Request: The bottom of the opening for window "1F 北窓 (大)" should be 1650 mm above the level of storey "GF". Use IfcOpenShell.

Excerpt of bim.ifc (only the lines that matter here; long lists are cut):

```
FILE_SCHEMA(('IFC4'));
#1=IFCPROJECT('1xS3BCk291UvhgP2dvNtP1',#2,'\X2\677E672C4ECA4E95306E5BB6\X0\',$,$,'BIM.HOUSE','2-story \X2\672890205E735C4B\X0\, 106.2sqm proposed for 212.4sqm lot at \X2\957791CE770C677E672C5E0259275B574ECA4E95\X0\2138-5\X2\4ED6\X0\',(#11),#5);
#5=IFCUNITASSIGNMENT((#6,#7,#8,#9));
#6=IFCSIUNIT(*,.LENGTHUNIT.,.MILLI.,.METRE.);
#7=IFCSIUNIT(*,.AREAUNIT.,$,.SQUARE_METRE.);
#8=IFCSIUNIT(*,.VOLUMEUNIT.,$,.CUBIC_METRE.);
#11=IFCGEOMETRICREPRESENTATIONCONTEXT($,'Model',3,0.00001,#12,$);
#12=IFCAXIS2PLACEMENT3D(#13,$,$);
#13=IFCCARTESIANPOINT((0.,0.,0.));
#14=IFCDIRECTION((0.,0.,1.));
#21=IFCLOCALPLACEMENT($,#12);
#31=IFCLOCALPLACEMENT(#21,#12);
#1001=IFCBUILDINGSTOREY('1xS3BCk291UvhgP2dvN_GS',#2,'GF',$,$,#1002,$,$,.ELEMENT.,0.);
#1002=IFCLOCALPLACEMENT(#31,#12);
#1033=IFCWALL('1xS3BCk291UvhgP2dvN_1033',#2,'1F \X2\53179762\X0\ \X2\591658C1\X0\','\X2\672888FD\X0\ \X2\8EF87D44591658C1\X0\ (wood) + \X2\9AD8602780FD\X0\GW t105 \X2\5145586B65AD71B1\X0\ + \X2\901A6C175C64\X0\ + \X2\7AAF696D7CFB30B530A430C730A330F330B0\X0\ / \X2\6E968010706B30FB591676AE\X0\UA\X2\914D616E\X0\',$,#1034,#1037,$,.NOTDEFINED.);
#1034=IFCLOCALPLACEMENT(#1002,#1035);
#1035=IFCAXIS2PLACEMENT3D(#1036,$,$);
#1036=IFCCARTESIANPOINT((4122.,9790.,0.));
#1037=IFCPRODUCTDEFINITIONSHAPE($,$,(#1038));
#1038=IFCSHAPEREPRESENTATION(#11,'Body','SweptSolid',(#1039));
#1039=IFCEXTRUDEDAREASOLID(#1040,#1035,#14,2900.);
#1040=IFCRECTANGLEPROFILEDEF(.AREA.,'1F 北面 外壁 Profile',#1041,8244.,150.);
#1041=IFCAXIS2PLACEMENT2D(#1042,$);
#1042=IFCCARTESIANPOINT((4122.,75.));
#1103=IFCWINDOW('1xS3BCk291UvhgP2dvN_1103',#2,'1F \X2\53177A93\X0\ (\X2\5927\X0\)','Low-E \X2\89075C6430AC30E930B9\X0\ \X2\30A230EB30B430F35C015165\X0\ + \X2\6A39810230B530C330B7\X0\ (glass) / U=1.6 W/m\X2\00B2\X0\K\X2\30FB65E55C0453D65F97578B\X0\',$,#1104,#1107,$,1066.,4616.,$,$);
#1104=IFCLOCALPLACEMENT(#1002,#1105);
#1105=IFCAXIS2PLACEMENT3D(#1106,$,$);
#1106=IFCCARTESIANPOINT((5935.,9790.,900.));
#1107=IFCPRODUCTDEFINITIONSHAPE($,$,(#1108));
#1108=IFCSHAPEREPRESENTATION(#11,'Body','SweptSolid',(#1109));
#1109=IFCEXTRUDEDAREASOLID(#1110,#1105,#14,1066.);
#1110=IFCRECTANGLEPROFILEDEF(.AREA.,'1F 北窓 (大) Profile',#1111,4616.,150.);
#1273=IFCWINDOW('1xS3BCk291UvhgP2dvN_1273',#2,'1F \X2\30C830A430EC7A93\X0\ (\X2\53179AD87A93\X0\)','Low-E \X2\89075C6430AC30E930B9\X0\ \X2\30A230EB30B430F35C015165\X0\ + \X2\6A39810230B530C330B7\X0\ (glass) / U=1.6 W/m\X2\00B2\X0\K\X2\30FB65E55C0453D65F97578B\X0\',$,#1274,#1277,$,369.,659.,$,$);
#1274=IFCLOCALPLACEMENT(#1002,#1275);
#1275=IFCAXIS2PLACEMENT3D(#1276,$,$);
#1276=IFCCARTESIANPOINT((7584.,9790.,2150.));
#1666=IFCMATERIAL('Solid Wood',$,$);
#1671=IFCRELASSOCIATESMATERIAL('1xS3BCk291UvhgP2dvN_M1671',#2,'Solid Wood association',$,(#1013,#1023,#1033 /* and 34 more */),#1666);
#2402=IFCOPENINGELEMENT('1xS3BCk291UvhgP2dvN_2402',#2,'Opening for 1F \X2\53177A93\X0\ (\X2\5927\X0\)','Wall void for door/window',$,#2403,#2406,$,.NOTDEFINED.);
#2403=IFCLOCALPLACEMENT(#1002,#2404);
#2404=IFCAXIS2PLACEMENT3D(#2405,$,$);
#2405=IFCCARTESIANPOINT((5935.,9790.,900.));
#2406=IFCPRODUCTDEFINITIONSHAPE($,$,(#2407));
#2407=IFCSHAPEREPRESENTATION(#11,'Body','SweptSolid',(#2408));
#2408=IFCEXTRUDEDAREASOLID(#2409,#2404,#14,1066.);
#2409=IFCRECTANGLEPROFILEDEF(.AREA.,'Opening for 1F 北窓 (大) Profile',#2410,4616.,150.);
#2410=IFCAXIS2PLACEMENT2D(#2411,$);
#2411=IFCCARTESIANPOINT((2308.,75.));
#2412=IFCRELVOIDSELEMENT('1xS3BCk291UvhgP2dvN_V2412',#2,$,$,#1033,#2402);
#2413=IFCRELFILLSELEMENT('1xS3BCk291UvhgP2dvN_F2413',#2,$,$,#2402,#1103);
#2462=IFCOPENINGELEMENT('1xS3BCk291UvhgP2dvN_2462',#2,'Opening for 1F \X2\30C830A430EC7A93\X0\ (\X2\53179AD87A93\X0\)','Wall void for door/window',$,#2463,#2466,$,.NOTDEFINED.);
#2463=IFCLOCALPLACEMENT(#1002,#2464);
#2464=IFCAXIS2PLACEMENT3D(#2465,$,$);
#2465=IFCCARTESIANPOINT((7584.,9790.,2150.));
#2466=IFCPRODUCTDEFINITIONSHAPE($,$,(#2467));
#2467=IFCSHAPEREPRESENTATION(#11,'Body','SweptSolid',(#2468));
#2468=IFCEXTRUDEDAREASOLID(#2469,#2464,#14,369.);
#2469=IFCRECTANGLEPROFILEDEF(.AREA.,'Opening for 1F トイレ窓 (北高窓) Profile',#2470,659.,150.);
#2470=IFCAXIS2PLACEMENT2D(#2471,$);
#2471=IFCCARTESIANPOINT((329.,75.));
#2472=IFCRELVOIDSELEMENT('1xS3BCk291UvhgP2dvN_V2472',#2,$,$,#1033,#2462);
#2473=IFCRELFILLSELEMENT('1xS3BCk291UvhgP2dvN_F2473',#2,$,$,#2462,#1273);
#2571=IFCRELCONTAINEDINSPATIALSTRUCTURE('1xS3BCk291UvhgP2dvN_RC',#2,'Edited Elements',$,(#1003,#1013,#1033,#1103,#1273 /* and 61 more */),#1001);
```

```python
import numpy as np
import ifcopenshell
import ifcopenshell.api.geometry
import ifcopenshell.geom
import ifcopenshell.util.element
import ifcopenshell.util.placement
import ifcopenshell.util.shape
import ifcopenshell.util.unit

model = ifcopenshell.open("bim.ifc")
unit_scale = ifcopenshell.util.unit.calculate_unit_scale(model)

window = model.by_id(1103)
opening = window.FillsVoids[0].RelatingOpeningElement
storey = ifcopenshell.util.element.get_container(window, ifc_class="IfcBuildingStorey")
level = ifcopenshell.util.placement.get_local_placement(storey.ObjectPlacement)[2, 3]

# The opening's origin need not be at the sill, so measure its lowest point.
shape = ifcopenshell.geom.create_shape(ifcopenshell.geom.settings(), opening)
bottom = ifcopenshell.util.shape.get_shape_bottom_elevation(shape, shape.geometry) / unit_scale
dz = level + 1.65 / unit_scale - bottom

shift = np.array([0.0, 0.0, dz])
# The window is not placed relative to its opening, so move both.
for product in (opening, window):
    matrix = ifcopenshell.util.placement.get_local_placement(product.ObjectPlacement)
    matrix[:3, 3] += shift
    ifcopenshell.api.geometry.edit_object_placement(model, product=product, matrix=matrix, is_si=False)

print(f"moved by {dz * unit_scale:+.3f} m")

model.write("bim-out.ifc")
```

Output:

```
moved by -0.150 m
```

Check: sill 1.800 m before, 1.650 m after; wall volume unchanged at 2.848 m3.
